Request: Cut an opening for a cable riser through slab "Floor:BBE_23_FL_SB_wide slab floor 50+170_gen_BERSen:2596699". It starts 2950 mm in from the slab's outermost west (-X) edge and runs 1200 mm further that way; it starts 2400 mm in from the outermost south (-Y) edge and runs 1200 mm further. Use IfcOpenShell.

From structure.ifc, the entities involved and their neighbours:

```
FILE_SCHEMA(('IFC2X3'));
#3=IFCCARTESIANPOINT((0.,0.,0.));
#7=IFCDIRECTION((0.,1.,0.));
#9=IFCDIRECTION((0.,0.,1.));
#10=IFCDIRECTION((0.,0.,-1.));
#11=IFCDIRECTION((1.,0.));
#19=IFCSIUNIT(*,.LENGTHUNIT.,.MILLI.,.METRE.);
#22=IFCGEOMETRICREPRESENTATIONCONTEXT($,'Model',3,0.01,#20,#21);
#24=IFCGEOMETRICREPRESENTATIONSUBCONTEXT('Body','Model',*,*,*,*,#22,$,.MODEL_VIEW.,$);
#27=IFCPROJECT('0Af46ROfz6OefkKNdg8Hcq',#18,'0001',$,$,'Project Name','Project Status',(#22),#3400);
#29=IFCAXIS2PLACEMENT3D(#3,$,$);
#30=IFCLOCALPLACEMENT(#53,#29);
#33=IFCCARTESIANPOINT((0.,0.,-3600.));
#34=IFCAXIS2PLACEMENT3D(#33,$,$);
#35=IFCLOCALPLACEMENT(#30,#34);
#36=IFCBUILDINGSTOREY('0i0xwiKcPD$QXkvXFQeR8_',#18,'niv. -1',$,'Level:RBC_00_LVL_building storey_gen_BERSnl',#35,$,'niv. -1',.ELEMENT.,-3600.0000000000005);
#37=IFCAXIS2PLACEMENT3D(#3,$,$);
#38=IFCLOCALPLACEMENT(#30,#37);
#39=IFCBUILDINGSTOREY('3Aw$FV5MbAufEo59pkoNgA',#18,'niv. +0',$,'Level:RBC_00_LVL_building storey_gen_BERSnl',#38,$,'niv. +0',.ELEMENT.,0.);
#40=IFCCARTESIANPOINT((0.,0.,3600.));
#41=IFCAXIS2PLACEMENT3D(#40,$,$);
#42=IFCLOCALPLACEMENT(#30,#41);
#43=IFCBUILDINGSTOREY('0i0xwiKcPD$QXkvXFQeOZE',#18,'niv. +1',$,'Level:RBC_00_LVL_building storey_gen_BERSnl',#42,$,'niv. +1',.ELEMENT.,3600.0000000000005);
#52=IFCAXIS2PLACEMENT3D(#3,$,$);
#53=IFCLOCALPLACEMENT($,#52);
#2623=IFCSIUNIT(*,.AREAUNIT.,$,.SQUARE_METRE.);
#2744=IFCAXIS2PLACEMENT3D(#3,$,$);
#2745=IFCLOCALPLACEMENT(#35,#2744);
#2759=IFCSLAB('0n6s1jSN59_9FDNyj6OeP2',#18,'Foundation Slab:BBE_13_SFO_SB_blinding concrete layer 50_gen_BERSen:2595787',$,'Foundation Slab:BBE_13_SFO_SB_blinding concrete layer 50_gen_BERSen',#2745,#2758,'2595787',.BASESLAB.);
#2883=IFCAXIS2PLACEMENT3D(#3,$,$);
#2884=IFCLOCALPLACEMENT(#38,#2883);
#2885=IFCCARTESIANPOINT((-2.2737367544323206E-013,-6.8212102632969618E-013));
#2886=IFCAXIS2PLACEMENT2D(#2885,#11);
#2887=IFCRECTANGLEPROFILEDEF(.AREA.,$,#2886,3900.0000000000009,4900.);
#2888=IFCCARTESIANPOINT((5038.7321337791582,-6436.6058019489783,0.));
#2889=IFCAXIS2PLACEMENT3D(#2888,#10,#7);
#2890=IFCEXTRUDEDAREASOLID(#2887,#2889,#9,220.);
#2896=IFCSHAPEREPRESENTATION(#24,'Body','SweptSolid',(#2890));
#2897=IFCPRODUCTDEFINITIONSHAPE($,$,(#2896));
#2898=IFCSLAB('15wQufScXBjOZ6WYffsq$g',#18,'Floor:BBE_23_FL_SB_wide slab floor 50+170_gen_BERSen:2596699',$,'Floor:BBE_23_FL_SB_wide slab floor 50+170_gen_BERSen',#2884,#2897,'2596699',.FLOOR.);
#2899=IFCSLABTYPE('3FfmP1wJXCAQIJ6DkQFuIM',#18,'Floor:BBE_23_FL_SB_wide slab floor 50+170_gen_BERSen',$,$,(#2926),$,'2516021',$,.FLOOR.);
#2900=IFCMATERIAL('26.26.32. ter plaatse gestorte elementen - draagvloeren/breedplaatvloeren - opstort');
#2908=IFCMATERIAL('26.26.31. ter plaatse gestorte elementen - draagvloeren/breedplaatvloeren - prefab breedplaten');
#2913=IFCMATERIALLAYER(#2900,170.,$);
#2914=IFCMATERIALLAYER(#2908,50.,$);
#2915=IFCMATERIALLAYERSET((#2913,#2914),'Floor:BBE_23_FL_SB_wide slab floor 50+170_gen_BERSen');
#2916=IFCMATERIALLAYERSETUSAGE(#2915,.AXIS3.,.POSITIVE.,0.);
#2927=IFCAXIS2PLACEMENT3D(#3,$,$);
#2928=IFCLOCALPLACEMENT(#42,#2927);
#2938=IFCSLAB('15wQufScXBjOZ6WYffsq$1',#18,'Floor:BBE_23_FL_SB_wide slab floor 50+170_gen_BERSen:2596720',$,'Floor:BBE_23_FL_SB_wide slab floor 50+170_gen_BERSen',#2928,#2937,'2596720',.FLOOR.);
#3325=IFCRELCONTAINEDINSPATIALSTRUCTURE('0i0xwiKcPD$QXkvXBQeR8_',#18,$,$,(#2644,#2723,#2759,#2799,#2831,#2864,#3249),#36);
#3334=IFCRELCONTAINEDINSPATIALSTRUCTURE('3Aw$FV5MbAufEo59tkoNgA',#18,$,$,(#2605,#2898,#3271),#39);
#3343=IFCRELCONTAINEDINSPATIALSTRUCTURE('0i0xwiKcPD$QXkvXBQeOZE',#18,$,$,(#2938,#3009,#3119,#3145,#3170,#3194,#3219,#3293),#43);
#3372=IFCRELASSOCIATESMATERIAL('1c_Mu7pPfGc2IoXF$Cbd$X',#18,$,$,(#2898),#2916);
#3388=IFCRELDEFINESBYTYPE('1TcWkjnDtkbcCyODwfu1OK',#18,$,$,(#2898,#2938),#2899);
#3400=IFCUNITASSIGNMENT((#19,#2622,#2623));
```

```python
import numpy as np
import ifcopenshell
import ifcopenshell.api.feature
import ifcopenshell.api.geometry
import ifcopenshell.api.root
import ifcopenshell.geom
import ifcopenshell.util.placement
import ifcopenshell.util.representation
import ifcopenshell.util.shape
import ifcopenshell.util.unit

model = ifcopenshell.open("structure.ifc")
unit_scale = ifcopenshell.util.unit.calculate_unit_scale(model)
settings = ifcopenshell.geom.settings()


def volume(element):
    """Net volume in cubic metres, openings subtracted."""
    shape = ifcopenshell.geom.create_shape(settings, element)
    return ifcopenshell.util.shape.get_volume(shape.geometry)


slab = model.by_guid("15wQufScXBjOZ6WYffsq$g")
before = volume(slab)

# Extent in the slab's own axes, in metres. The edges named are its -X and -Y sides.
slab_shape = ifcopenshell.geom.create_shape(settings, slab)
vertices = ifcopenshell.util.shape.get_vertices(slab_shape.geometry)
x_min, y_min, bottom = vertices.min(axis=0)
top = vertices[:, 2].max()

opening = ifcopenshell.api.root.create_entity(model, ifc_class="IfcOpeningElement", name="Cable riser opening")
context = ifcopenshell.util.representation.get_context(model, "Model", "Body", "MODEL_VIEW")
width, depth = 1.2, 1.2
outline = [(0.0, 0.0), (width, 0.0), (width, depth), (0.0, depth), (0.0, 0.0)]
# Overshoot both faces by 50 mm so the cut is clean.
shape = ifcopenshell.api.geometry.add_slab_representation(
    model, context=context, depth=top - bottom + 0.1, polyline=outline
)
ifcopenshell.api.geometry.assign_representation(model, product=opening, representation=shape)

matrix = ifcopenshell.util.placement.get_local_placement(slab.ObjectPlacement)
matrix[:, 3] = matrix @ np.append(np.array([x_min + 2.95, y_min + 2.4, bottom - 0.05]) / unit_scale, 1.0)
ifcopenshell.api.geometry.edit_object_placement(model, product=opening, matrix=matrix, is_si=False)
ifcopenshell.api.feature.add_feature(model, feature=opening, element=slab)

after = volume(slab)

print(f"slab volume {before:.3f} -> {after:.3f} m3")

model.write("structure_edited.ifc")
```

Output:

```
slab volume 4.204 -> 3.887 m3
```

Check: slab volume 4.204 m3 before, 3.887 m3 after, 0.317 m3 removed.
